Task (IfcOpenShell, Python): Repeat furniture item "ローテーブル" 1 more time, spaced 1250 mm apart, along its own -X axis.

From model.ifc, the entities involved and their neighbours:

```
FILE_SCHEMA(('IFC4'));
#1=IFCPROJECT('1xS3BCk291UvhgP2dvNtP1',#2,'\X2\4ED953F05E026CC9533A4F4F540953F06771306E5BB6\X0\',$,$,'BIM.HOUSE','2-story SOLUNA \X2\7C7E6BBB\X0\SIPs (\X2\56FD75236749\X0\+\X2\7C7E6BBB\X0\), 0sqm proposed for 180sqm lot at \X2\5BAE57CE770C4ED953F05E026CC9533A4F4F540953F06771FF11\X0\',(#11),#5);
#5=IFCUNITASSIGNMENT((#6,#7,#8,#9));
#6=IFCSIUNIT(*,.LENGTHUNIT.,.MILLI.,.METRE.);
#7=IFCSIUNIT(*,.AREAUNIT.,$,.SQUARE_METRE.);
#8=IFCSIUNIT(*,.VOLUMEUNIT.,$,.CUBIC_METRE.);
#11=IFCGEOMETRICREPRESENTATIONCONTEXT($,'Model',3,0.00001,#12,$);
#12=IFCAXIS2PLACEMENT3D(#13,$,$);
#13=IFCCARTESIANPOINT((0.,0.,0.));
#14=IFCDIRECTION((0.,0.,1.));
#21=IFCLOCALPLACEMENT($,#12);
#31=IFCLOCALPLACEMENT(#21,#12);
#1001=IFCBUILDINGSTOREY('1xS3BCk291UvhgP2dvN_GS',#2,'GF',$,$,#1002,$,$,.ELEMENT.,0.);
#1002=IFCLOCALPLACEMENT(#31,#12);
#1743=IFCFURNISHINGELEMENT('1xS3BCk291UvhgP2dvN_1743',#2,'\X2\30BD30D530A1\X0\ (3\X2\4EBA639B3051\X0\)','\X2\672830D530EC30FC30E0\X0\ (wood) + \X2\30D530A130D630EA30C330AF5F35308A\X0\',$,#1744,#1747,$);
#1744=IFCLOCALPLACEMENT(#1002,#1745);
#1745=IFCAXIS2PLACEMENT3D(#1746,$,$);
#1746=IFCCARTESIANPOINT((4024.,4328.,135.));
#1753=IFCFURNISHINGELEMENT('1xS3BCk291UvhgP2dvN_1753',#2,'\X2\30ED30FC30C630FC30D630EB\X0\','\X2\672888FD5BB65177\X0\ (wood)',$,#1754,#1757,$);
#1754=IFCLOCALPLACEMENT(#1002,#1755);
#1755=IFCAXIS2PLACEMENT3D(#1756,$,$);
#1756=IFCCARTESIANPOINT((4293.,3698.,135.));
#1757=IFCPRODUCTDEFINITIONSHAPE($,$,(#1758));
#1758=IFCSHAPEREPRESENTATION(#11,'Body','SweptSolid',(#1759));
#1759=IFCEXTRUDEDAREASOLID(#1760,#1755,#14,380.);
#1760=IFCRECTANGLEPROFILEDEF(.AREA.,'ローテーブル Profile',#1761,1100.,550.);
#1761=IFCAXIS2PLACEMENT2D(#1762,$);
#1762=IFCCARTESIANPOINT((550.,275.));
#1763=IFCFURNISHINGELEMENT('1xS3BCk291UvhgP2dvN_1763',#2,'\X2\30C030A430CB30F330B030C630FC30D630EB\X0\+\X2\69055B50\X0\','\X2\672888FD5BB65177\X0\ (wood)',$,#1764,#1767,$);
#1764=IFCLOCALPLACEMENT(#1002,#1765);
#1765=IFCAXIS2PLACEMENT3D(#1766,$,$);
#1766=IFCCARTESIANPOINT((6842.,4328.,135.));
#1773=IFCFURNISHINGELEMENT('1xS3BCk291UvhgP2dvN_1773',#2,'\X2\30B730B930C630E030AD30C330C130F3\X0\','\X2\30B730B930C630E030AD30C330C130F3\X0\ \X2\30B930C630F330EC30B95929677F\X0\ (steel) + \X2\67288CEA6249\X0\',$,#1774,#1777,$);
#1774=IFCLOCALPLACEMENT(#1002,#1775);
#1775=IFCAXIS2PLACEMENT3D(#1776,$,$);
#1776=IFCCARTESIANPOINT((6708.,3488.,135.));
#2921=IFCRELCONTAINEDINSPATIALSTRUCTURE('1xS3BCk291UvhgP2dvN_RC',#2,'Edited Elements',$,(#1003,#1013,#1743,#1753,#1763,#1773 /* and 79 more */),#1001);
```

```python
import ifcopenshell
import ifcopenshell.api.geometry
import ifcopenshell.api.root
import ifcopenshell.util.element
import ifcopenshell.util.placement
import ifcopenshell.util.unit

model = ifcopenshell.open("model.ifc")
unit_scale = ifcopenshell.util.unit.calculate_unit_scale(model)


def reuse_history(source, copy):
    """copy_class also copies each property set's owner history, people and application; keep the originals."""
    for rel in copy.IsDefinedBy:
        if rel.is_a("IfcRelDefinesByProperties") and (history := rel.RelatingPropertyDefinition.OwnerHistory):
            rel.RelatingPropertyDefinition.OwnerHistory = source.OwnerHistory
            ifcopenshell.util.element.remove_deep2(model, history)


source = model.by_guid("1xS3BCk291UvhgP2dvN_1753")
base = ifcopenshell.util.placement.get_local_placement(source.ObjectPlacement)
step = -base[:3, 0] * 1.25 / unit_scale

for i in range(1, 2):
    copy = ifcopenshell.api.root.copy_class(model, product=source)
    copy.Representation = ifcopenshell.util.element.copy_deep(
        model, source.Representation, exclude=["IfcGeometricRepresentationContext", "IfcRepresentationMap"]
    )
    reuse_history(source, copy)
    matrix = base.copy()
    matrix[:3, 3] += i * step
    print("added at", matrix[:3, 3].round(3) + 0.0)
    ifcopenshell.api.geometry.edit_object_placement(model, product=copy, matrix=matrix, is_si=False)

model.write("model_v2.ifc")
```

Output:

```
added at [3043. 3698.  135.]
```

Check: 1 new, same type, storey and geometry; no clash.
